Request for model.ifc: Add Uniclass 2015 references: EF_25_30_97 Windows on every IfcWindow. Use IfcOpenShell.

First a look at what the model holds.

```python
import ifcopenshell

model = ifcopenshell.open("model.ifc")
print(model.schema)
print("classifications:", [c.Name for c in model.by_type("IfcClassification")])
for ifc_class in ("IfcDoor", "IfcRoof", "IfcStair", "IfcWall", "IfcWindow"):
    print(ifc_class, len(model.by_type(ifc_class)))
```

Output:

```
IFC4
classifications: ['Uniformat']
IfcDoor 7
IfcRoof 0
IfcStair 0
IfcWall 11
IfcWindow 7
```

```python
import ifcopenshell
import ifcopenshell.api.classification

model = ifcopenshell.open("model.ifc")

system = ifcopenshell.api.classification.add_classification(model, classification="Uniclass 2015")

codes = {
    "IfcWindow": ("EF_25_30_97", "Windows"),
}
for ifc_class, (code, name) in codes.items():
    products = model.by_type(ifc_class)
    ifcopenshell.api.classification.add_reference(
        model, products=products, classification=system, identification=code, name=name
    )
    print(code, len(products))

model.write("model_edited.ifc")
```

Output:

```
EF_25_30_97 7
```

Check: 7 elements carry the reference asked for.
